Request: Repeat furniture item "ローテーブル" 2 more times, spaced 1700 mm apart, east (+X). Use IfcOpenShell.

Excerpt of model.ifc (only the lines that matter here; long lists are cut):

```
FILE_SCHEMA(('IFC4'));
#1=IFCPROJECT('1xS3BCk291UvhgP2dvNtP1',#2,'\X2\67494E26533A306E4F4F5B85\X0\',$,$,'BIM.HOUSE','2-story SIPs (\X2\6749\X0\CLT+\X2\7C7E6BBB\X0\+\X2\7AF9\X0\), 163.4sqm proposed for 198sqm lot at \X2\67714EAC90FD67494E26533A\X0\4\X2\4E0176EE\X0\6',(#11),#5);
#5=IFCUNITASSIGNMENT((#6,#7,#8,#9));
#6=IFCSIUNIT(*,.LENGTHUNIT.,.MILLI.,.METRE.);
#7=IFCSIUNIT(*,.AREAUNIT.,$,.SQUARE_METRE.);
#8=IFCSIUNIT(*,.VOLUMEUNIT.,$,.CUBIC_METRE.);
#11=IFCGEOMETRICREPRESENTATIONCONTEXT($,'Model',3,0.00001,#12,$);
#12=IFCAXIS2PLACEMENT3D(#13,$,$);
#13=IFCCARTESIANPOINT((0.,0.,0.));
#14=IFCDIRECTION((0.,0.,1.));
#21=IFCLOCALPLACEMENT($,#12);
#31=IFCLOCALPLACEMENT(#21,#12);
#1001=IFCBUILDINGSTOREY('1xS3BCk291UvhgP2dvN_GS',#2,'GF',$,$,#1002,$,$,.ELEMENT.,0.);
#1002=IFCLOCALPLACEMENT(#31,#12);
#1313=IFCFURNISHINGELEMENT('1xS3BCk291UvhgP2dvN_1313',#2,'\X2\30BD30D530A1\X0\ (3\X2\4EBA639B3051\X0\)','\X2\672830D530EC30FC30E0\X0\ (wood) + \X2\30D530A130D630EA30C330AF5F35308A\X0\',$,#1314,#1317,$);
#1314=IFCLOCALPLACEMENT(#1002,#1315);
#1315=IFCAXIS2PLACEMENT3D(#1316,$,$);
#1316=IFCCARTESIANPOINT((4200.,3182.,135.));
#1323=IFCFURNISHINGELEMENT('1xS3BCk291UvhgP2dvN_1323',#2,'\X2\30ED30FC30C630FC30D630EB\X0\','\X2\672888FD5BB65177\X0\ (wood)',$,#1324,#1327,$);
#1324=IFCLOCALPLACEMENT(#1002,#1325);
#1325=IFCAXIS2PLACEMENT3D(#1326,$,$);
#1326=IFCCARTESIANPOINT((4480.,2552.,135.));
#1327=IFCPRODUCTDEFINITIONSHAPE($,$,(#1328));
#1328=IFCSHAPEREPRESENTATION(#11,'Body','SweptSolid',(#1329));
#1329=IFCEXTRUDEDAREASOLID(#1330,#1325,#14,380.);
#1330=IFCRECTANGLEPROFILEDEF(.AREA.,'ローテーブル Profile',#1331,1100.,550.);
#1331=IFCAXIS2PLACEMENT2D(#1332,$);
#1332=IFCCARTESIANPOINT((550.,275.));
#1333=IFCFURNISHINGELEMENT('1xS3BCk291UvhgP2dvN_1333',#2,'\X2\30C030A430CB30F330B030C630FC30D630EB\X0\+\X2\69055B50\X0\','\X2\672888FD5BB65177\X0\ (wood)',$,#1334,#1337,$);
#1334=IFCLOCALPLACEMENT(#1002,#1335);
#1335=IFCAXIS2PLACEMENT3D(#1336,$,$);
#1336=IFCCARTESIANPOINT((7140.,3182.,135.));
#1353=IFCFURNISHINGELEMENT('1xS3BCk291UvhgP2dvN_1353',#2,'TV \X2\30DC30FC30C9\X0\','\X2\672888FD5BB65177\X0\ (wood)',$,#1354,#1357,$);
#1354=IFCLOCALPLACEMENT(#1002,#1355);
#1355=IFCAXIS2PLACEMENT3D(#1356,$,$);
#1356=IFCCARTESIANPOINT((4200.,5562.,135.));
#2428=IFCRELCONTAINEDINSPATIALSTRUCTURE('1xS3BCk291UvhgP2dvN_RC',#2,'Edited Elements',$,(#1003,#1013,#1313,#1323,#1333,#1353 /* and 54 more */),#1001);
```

```python
import numpy as np
import ifcopenshell
import ifcopenshell.api.geometry
import ifcopenshell.api.root
import ifcopenshell.util.element
import ifcopenshell.util.placement
import ifcopenshell.util.unit

model = ifcopenshell.open("model.ifc")
unit_scale = ifcopenshell.util.unit.calculate_unit_scale(model)


def reuse_history(source, copy):
    """copy_class also copies each property set's owner history, people and application; keep the originals."""
    for rel in copy.IsDefinedBy:
        if rel.is_a("IfcRelDefinesByProperties") and (history := rel.RelatingPropertyDefinition.OwnerHistory):
            rel.RelatingPropertyDefinition.OwnerHistory = source.OwnerHistory
            ifcopenshell.util.element.remove_deep2(model, history)


source = model.by_guid("1xS3BCk291UvhgP2dvN_1323")
base = ifcopenshell.util.placement.get_local_placement(source.ObjectPlacement)
step = np.array([1.0, 0.0, 0.0]) * 1.7 / unit_scale

for i in range(1, 3):
    copy = ifcopenshell.api.root.copy_class(model, product=source)
    copy.Representation = ifcopenshell.util.element.copy_deep(
        model, source.Representation, exclude=["IfcGeometricRepresentationContext", "IfcRepresentationMap"]
    )
    reuse_history(source, copy)
    matrix = base.copy()
    matrix[:3, 3] += i * step
    print("added at", matrix[:3, 3].round(3) + 0.0)
    ifcopenshell.api.geometry.edit_object_placement(model, product=copy, matrix=matrix, is_si=False)

model.write("model_rev.ifc")
```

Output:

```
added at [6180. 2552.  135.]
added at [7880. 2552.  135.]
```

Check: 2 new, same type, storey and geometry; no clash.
